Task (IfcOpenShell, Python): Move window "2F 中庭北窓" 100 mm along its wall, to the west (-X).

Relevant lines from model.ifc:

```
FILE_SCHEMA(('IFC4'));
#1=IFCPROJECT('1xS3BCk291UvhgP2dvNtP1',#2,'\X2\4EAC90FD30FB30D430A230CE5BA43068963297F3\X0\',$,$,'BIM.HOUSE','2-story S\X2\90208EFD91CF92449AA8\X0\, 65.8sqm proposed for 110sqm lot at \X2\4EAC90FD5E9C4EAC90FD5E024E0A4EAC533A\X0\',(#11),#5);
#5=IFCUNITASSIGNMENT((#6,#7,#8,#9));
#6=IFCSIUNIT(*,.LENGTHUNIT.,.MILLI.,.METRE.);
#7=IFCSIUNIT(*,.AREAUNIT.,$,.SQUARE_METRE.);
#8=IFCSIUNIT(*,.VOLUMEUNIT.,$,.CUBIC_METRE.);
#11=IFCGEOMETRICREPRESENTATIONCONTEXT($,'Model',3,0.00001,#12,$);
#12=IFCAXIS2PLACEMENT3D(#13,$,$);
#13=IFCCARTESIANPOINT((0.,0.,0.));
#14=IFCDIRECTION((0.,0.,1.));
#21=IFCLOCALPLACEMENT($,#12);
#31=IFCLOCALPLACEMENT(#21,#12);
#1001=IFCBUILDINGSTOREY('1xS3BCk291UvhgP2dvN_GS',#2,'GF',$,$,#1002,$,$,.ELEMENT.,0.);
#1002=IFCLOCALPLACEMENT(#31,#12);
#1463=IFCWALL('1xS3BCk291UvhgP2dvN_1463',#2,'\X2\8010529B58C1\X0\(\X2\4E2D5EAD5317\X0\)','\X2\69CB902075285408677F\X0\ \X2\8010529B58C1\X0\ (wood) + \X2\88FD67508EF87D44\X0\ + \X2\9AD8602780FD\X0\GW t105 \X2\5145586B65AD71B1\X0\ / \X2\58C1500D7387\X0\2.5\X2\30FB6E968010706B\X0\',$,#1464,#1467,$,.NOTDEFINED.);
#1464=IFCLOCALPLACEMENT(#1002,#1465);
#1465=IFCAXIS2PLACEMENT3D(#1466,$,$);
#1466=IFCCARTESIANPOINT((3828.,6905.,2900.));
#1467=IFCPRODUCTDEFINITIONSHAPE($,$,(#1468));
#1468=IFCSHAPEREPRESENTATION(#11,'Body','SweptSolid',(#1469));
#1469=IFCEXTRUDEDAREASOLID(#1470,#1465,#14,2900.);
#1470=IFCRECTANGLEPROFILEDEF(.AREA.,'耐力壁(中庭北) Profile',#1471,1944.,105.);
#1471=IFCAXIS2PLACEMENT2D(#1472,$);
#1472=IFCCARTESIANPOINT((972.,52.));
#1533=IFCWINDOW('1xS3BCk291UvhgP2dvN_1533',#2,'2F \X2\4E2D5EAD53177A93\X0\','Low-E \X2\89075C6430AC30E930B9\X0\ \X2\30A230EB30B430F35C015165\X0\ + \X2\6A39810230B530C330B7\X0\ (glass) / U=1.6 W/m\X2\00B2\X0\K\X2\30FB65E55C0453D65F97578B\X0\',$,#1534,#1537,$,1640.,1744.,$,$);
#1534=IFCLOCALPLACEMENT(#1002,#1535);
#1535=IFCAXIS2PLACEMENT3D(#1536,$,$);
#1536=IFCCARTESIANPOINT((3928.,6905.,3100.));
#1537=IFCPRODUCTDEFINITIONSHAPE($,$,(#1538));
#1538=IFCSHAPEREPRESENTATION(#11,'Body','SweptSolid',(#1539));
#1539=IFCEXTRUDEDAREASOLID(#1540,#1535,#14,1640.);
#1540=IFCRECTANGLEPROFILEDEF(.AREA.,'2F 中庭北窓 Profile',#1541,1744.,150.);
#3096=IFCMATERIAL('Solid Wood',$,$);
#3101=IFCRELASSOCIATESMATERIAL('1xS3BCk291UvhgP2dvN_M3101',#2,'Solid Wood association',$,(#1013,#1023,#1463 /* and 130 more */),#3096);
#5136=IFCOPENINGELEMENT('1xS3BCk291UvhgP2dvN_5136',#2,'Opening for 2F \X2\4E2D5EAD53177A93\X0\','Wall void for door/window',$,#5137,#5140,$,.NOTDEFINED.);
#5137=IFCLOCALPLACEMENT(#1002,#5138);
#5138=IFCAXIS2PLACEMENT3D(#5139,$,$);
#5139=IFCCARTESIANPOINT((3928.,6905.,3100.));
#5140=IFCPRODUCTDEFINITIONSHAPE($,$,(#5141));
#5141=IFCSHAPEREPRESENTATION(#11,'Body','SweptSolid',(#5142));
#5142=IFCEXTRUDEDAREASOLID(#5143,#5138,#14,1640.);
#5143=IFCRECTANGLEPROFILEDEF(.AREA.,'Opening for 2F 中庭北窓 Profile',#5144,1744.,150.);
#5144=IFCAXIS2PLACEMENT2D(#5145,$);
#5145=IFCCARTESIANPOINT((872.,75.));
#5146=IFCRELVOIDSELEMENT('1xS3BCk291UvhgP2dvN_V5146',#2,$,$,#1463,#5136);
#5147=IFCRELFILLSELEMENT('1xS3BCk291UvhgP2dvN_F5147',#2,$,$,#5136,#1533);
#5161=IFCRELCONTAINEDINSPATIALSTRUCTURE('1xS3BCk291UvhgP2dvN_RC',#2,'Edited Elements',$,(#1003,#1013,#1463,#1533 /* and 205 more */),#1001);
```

```python
import ifcopenshell
import ifcopenshell.api.geometry
import ifcopenshell.util.placement

model = ifcopenshell.open("model.ifc")

window = model.by_id(1533)
opening = window.FillsVoids[0].RelatingOpeningElement
wall = opening.VoidsElements[0].RelatingBuildingElement

wall_matrix = ifcopenshell.util.placement.get_local_placement(wall.ObjectPlacement)
shift = wall_matrix[:3, 0] * -100.0
before = ifcopenshell.util.placement.get_local_placement(window.ObjectPlacement)[:3, 3].copy()

# The window is not placed relative to its opening, so move both.
for product in (opening, window):
    matrix = ifcopenshell.util.placement.get_local_placement(product.ObjectPlacement)
    matrix[:3, 3] += shift
    ifcopenshell.api.geometry.edit_object_placement(model, product=product, matrix=matrix, is_si=False)

after = ifcopenshell.util.placement.get_local_placement(window.ObjectPlacement)[:3, 3]
print("window moved by", (after - before).round(3) + 0.0)

model.write("model_v2.ifc")
```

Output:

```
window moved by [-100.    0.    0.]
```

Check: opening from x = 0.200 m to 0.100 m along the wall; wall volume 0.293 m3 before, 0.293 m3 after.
